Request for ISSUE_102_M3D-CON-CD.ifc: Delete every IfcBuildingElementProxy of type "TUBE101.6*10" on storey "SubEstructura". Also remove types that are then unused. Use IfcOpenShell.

First a look at what the model holds.

```python
import ifcopenshell
import ifcopenshell.util.element

model = ifcopenshell.open("ISSUE_102_M3D-CON-CD.ifc")
print(model.schema)
storey = next(s for s in model.by_type("IfcBuildingStorey") if s.Name == "SubEstructura")
proxies = [e for e in ifcopenshell.util.element.get_decomposition(storey) if e.is_a("IfcBuildingElementProxy")]
seen = {}
for e in proxies:
    element_type = ifcopenshell.util.element.get_type(e)
    name = element_type.Name if element_type not in (None, e) else None
    seen[name] = seen.get(name, 0) + 1
for name, count in sorted(seen.items(), key=str):
    print(count, "x", name)
```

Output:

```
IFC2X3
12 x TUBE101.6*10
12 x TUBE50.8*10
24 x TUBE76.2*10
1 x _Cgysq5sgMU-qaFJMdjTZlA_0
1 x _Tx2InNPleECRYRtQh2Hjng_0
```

```python
import ifcopenshell
import ifcopenshell.api.root
import ifcopenshell.util.element

model = ifcopenshell.open("ISSUE_102_M3D-CON-CD.ifc")

storey = next(s for s in model.by_type("IfcBuildingStorey") if s.Name == "SubEstructura")
proxies = [e for e in ifcopenshell.util.element.get_decomposition(storey) if e.is_a("IfcBuildingElementProxy")]
targets = [e for e in proxies if (t := ifcopenshell.util.element.get_type(e)) not in (None, e) and t.Name == "TUBE101.6*10"]
types = {ifcopenshell.util.element.get_type(e) for e in targets} - {None, *targets}

for e in targets:
    ifcopenshell.api.root.remove_product(model, product=e)
print(len(targets), "removed")

unused = [t for t in types if not ifcopenshell.util.element.get_types(t)]
for t in unused:
    ifcopenshell.api.root.remove_product(model, product=t)
print(len(unused), "unused types removed")

model.write("ISSUE_102_M3D-CON-CD_rev.ifc")
```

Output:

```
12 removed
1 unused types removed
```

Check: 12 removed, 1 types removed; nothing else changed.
